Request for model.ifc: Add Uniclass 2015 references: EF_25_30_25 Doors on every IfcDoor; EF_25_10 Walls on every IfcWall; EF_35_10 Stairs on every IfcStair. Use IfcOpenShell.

First a look at what the model holds.

```python
import ifcopenshell

model = ifcopenshell.open("model.ifc")
print(model.schema)
print("classifications:", [c.Name for c in model.by_type("IfcClassification")])
for ifc_class in ("IfcDoor", "IfcRoof", "IfcStair", "IfcWall", "IfcWindow"):
    print(ifc_class, len(model.by_type(ifc_class)))
```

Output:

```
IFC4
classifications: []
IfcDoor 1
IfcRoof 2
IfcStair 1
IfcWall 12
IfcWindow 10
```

```python
import ifcopenshell
import ifcopenshell.api.classification

model = ifcopenshell.open("model.ifc")

system = ifcopenshell.api.classification.add_classification(model, classification="Uniclass 2015")

codes = {
    "IfcDoor": ("EF_25_30_25", "Doors"),
    "IfcWall": ("EF_25_10", "Walls"),
    "IfcStair": ("EF_35_10", "Stairs"),
}
for ifc_class, (code, name) in codes.items():
    products = model.by_type(ifc_class)
    ifcopenshell.api.classification.add_reference(
        model, products=products, classification=system, identification=code, name=name
    )
    print(code, len(products))

model.write("model_updated.ifc")
```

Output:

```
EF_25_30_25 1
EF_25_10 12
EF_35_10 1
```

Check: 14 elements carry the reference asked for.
